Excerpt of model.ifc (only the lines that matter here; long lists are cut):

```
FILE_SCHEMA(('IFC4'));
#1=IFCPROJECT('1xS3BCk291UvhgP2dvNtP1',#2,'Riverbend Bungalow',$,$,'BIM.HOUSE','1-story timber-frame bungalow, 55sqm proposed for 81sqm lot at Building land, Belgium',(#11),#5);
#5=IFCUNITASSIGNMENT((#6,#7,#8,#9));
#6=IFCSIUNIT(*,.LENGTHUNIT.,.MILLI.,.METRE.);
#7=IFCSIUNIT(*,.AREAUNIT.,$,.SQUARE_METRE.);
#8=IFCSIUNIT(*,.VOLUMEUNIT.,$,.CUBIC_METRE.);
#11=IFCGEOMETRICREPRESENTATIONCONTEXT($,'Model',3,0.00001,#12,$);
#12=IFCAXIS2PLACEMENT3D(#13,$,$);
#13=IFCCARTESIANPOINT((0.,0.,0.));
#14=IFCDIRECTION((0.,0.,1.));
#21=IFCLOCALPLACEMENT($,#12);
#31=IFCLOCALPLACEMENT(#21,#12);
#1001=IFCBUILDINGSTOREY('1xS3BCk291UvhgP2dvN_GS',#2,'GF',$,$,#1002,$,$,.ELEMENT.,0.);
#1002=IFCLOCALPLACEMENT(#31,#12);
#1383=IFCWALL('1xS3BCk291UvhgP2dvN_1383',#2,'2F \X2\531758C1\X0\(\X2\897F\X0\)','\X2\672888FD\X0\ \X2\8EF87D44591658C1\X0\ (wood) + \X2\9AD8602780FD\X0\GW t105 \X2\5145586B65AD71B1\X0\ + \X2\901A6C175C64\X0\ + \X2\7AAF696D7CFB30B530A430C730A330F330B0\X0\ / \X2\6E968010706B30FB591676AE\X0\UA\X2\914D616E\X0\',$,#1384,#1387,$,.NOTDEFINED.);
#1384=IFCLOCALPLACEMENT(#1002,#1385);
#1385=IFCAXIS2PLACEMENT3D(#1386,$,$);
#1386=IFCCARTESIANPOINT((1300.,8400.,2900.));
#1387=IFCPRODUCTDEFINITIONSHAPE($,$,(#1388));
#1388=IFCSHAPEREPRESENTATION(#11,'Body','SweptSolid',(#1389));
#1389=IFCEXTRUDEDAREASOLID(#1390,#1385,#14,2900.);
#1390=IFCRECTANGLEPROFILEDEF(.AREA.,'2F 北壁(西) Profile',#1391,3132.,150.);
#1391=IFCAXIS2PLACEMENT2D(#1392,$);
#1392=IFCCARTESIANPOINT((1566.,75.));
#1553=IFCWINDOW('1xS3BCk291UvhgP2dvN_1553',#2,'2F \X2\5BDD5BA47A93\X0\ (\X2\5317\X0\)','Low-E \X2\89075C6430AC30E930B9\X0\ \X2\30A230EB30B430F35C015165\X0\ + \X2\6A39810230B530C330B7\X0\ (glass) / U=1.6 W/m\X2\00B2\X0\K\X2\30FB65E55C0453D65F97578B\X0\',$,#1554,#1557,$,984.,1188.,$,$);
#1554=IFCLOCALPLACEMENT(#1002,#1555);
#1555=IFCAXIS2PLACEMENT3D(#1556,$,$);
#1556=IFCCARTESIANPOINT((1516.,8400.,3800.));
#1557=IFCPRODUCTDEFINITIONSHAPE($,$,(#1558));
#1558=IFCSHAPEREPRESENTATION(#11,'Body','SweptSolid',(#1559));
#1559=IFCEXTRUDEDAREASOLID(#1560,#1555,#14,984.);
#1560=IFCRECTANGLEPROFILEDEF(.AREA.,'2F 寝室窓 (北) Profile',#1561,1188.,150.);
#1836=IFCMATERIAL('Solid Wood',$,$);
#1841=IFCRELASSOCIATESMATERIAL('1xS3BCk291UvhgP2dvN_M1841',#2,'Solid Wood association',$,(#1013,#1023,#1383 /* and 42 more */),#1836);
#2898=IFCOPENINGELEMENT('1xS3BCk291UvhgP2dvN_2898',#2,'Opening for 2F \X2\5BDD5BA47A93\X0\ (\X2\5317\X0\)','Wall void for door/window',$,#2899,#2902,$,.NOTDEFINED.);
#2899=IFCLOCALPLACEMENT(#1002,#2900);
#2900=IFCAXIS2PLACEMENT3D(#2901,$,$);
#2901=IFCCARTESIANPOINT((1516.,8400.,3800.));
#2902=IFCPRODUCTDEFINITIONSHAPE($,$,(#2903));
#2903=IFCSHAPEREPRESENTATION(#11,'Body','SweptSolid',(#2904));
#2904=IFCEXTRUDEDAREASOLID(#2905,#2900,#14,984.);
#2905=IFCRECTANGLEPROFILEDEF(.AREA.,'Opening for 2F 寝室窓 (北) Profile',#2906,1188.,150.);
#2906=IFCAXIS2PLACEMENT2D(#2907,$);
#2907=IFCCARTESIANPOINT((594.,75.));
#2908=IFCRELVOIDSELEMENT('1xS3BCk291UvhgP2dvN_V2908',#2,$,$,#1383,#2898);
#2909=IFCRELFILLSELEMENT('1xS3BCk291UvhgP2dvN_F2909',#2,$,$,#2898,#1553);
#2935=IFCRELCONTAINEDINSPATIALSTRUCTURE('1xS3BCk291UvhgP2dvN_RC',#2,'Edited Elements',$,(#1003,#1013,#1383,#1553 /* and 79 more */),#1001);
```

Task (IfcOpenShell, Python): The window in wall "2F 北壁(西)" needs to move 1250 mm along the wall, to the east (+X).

```python
import ifcopenshell
import ifcopenshell.api.geometry
import ifcopenshell.util.placement
import ifcopenshell.util.unit

model = ifcopenshell.open("model.ifc")
unit_scale = ifcopenshell.util.unit.calculate_unit_scale(model)

window = model.by_id(1553)
opening = window.FillsVoids[0].RelatingOpeningElement
wall = opening.VoidsElements[0].RelatingBuildingElement

wall_matrix = ifcopenshell.util.placement.get_local_placement(wall.ObjectPlacement)
shift = wall_matrix[:3, 0] * 1.25 / unit_scale
before = ifcopenshell.util.placement.get_local_placement(window.ObjectPlacement)[:3, 3].copy()

# The window is not placed relative to its opening, so move both.
for product in (opening, window):
    matrix = ifcopenshell.util.placement.get_local_placement(product.ObjectPlacement)
    matrix[:3, 3] += shift
    ifcopenshell.api.geometry.edit_object_placement(model, product=product, matrix=matrix, is_si=False)

after = ifcopenshell.util.placement.get_local_placement(window.ObjectPlacement)[:3, 3]
print("window moved by", (after - before).round(3) + 0.0)

model.write("model_updated.ifc")
```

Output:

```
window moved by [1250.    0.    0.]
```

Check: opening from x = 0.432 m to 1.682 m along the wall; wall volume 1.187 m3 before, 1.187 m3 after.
